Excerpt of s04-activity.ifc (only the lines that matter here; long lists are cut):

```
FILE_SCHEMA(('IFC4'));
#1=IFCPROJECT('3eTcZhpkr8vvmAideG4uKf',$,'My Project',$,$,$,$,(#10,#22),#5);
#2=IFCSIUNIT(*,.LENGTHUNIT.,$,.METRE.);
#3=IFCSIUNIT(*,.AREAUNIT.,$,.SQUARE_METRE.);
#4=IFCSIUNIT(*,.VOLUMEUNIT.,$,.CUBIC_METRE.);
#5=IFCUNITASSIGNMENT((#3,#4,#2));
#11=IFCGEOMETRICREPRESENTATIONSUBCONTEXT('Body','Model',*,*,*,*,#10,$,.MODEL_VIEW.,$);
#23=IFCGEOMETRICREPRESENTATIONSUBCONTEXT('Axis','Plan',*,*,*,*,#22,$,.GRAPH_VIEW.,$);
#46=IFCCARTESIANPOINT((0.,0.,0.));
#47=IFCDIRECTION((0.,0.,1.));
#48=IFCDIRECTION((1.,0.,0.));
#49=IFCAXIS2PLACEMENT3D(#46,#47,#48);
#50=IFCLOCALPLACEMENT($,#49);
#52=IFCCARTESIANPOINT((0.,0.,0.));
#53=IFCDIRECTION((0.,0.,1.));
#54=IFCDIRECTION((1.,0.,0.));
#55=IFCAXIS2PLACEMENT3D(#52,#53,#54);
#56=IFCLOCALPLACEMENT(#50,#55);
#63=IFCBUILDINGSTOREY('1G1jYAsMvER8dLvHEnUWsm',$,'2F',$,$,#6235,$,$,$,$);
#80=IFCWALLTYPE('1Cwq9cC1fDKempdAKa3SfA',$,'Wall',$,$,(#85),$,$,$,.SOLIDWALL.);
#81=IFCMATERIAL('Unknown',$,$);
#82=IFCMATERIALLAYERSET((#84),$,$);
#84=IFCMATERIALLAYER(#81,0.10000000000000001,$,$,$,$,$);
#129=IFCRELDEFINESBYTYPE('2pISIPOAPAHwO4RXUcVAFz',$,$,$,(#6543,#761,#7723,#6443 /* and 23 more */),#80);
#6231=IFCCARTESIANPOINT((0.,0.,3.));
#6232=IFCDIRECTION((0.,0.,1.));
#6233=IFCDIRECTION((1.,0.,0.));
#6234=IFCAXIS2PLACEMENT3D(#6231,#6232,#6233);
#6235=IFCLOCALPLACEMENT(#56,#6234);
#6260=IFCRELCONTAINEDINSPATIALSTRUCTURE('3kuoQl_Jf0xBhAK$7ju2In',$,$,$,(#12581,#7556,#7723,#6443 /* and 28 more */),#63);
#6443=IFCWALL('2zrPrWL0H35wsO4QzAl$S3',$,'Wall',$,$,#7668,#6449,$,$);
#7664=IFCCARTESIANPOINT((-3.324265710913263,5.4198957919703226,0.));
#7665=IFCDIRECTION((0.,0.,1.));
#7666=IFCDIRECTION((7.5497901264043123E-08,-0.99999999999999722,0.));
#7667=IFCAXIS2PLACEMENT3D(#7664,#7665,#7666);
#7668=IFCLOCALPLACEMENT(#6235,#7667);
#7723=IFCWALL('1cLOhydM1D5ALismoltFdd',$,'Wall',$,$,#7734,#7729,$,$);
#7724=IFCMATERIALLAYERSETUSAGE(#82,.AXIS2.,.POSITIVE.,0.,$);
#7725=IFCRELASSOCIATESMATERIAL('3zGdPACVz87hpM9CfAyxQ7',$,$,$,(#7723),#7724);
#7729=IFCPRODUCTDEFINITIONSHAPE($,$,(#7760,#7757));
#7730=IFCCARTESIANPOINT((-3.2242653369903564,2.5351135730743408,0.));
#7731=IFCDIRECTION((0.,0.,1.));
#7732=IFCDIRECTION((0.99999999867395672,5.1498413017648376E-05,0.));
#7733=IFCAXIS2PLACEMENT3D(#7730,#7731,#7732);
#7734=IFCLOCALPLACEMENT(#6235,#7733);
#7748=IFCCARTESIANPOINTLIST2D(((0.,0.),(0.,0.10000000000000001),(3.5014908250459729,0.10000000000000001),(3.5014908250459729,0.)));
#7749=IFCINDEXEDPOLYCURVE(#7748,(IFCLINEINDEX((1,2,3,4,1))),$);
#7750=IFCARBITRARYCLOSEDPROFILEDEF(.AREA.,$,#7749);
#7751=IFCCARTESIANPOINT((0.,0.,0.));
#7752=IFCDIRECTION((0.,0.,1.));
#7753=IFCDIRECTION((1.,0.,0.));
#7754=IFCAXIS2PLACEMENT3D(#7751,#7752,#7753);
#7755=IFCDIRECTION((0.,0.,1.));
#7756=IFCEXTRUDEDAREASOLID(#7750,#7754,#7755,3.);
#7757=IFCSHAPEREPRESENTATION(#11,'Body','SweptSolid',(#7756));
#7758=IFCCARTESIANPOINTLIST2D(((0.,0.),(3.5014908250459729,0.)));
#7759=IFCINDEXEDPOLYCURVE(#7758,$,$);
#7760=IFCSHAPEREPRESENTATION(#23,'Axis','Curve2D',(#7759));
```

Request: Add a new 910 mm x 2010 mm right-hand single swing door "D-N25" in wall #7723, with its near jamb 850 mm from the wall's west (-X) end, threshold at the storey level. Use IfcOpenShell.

```python
import numpy as np
import ifcopenshell
import ifcopenshell.api.feature
import ifcopenshell.api.geometry
import ifcopenshell.api.root
import ifcopenshell.api.spatial
import ifcopenshell.geom
import ifcopenshell.util.element
import ifcopenshell.util.placement
import ifcopenshell.util.representation
import ifcopenshell.util.shape
import ifcopenshell.util.unit

model = ifcopenshell.open("s04-activity.ifc")
unit_scale = ifcopenshell.util.unit.calculate_unit_scale(model)
settings = ifcopenshell.geom.settings()


def volume(element):
    """Net volume in cubic metres, openings subtracted."""
    shape = ifcopenshell.geom.create_shape(settings, element)
    return ifcopenshell.util.shape.get_volume(shape.geometry)


wall = model.by_guid("1cLOhydM1D5ALismoltFdd")
storey = ifcopenshell.util.element.get_container(wall, ifc_class="IfcBuildingStorey")
context = ifcopenshell.util.representation.get_context(model, "Model", "Body", "MODEL_VIEW")
before = volume(wall)

width, height, from_end, sill = 0.91, 2.01, 0.85, 0.0  # metres

# The wall runs along its own X axis, and the end named is its -X end.
wall_shape = ifcopenshell.geom.create_shape(settings, wall)
x, y, z = ifcopenshell.util.shape.get_vertices(wall_shape.geometry).T
start = x.min() + from_end
face, thickness = float(y.min()), float(y.max() - y.min())
wall_matrix = ifcopenshell.util.placement.get_local_placement(wall.ObjectPlacement)
level = ifcopenshell.util.placement.get_local_placement(storey.ObjectPlacement)[2, 3]


def in_wall(x, y):
    """Placement at x, y metres in the wall's axes, at sill height."""
    matrix = wall_matrix.copy()
    matrix[:, 3] = wall_matrix @ np.array([x / unit_scale, y / unit_scale, 0.0, 1.0])
    matrix[2, 3] = level + sill / unit_scale
    return matrix


# Opening: a box that overshoots both wall faces by 50 mm.
opening = ifcopenshell.api.root.create_entity(model, ifc_class="IfcOpeningElement", predefined_type="OPENING")
box = ifcopenshell.api.geometry.add_wall_representation(
    model, context=context, length=width, height=height, thickness=thickness + 0.1
)
ifcopenshell.api.geometry.assign_representation(model, product=opening, representation=box)
ifcopenshell.api.geometry.edit_object_placement(model, product=opening, matrix=in_wall(start, face - 0.05), is_si=False)
ifcopenshell.api.feature.add_feature(model, feature=opening, element=wall)

door = ifcopenshell.api.root.create_entity(model, ifc_class="IfcDoor", name="D-N25", predefined_type="DOOR")
door.OverallWidth, door.OverallHeight = width / unit_scale, height / unit_scale
door.OperationType = "SINGLE_SWING_RIGHT"
body = ifcopenshell.api.geometry.add_door_representation(
    model,
    context=context,
    overall_width=door.OverallWidth,
    overall_height=door.OverallHeight,
    operation_type="SINGLE_SWING_RIGHT",
    lining_properties={"LiningDepth": thickness / unit_scale, "ThresholdDepth": thickness / unit_scale},
)
ifcopenshell.api.geometry.assign_representation(model, product=door, representation=body)
ifcopenshell.api.spatial.assign_container(model, products=[door], relating_structure=storey)
ifcopenshell.api.feature.add_filling(model, opening=opening, element=door)

# The lining spans the wall, so the door starts at the wall face.
ifcopenshell.api.geometry.edit_object_placement(model, product=door, matrix=in_wall(start, face), is_si=False)

after = volume(wall)

print(f"wall volume {before:.3f} -> {after:.3f} m3")

model.write("s04-activity_updated.ifc")
```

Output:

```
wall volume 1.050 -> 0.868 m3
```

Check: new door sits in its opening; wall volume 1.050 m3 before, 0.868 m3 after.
